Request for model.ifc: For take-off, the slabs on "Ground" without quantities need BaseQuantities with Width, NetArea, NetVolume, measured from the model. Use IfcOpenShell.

First a look at what the model holds.

```python
import ifcopenshell
import ifcopenshell.util.element
import ifcopenshell.util.unit

model = ifcopenshell.open("model.ifc")
print(model.schema)
for unit_type in ("LENGTHUNIT", "AREAUNIT", "VOLUMEUNIT"):
    print(unit_type, ifcopenshell.util.unit.calculate_unit_scale(model, unit_type))
storey = next(s for s in model.by_type("IfcBuildingStorey") if s.Name == "Ground")
slabs = [e for e in ifcopenshell.util.element.get_decomposition(storey) if e.is_a("IfcSlab")]
for e in sorted(slabs, key=lambda e: e.id()):
    print(e.id(), e.is_a(), e.Name, list(ifcopenshell.util.element.get_psets(e, qtos_only=True)), sep=" | ")
```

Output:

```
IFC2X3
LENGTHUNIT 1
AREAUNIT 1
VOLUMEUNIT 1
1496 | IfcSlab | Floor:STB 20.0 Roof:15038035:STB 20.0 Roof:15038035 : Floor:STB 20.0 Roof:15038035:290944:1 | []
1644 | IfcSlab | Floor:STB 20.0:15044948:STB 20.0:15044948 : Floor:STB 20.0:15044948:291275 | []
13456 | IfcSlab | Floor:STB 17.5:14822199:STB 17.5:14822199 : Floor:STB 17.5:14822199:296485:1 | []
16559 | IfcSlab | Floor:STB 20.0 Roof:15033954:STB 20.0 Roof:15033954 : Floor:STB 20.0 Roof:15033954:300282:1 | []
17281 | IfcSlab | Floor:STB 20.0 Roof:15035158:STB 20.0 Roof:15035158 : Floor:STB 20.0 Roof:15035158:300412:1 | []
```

```python
import ifcopenshell
import ifcopenshell.api.pset
import ifcopenshell.geom
import ifcopenshell.util.element
import ifcopenshell.util.shape
import ifcopenshell.util.unit

model = ifcopenshell.open("model.ifc")
unit_scale = ifcopenshell.util.unit.calculate_unit_scale(model)
area_scale = ifcopenshell.util.unit.calculate_unit_scale(model, "AREAUNIT")
volume_scale = ifcopenshell.util.unit.calculate_unit_scale(model, "VOLUMEUNIT")
settings = ifcopenshell.geom.settings()

storey = next(s for s in model.by_type("IfcBuildingStorey") if s.Name == "Ground")
slabs = [e for e in ifcopenshell.util.element.get_decomposition(storey) if e.is_a("IfcSlab")]

for e in sorted(slabs, key=lambda e: e.id()):
    if ifcopenshell.util.element.get_psets(e, qtos_only=True, should_inherit=False):
        continue
    # Geometry comes back in metres, in the element's own axes.
    shape = ifcopenshell.geom.create_shape(settings, e)
    values = {
        "Width": ifcopenshell.util.shape.get_z(shape.geometry) / unit_scale,
        "NetArea": ifcopenshell.util.shape.get_footprint_area(shape.geometry) / area_scale,
        "NetVolume": ifcopenshell.util.shape.get_volume(shape.geometry) / volume_scale,
    }
    qto = ifcopenshell.api.pset.add_qto(model, product=e, name="BaseQuantities")
    ifcopenshell.api.pset.edit_qto(model, qto=qto, properties=values)
    print(e.id(), {k: round(v, 3) for k, v in values.items()})

model.write("model_updated.ifc")
```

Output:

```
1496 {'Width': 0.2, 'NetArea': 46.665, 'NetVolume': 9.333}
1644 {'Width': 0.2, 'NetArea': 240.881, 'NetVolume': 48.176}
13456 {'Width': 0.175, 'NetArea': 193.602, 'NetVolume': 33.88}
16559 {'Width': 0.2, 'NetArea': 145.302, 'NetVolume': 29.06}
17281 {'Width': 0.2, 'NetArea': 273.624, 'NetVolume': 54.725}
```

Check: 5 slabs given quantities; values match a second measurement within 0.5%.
